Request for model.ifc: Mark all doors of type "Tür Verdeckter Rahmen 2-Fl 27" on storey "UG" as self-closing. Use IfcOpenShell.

First a look at what the model holds.

```python
import ifcopenshell
import ifcopenshell.util.element

model = ifcopenshell.open("model.ifc")
print(model.schema)
storey = next(s for s in model.by_type("IfcBuildingStorey") if s.Name == "UG")
doors = [e for e in ifcopenshell.util.element.get_decomposition(storey) if e.is_a("IfcDoor")]
seen = {}
for e in doors:
    element_type = ifcopenshell.util.element.get_type(e)
    key = (element_type.Name if element_type != e and element_type else None, ifcopenshell.util.element.get_pset(e, "Pset_DoorCommon", "SelfClosing"))
    seen[key] = seen.get(key, 0) + 1
for (name, value), count in sorted(seen.items(), key=str):
    print(count, "x", name, "|", value)
```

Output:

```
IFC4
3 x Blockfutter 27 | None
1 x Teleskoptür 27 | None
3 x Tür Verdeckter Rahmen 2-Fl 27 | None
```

```python
import ifcopenshell
import ifcopenshell.api.pset
import ifcopenshell.util.element

model = ifcopenshell.open("model.ifc")

storey = next(s for s in model.by_type("IfcBuildingStorey") if s.Name == "UG")
doors = [e for e in ifcopenshell.util.element.get_decomposition(storey) if e.is_a("IfcDoor")]

count = 0
for e in doors:
    element_type = ifcopenshell.util.element.get_type(e)
    if element_type in (None, e) or element_type.Name != "Tür Verdeckter Rahmen 2-Fl 27":
        continue
    # add_pset returns the element's existing set when there is one.
    pset = ifcopenshell.api.pset.add_pset(model, product=e, name="Pset_DoorCommon")
    ifcopenshell.api.pset.edit_pset(model, pset=pset, properties={"SelfClosing": True})
    count += 1

print(count, "doors updated")

model.write("model_v2.ifc")
```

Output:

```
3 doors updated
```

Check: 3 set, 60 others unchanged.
